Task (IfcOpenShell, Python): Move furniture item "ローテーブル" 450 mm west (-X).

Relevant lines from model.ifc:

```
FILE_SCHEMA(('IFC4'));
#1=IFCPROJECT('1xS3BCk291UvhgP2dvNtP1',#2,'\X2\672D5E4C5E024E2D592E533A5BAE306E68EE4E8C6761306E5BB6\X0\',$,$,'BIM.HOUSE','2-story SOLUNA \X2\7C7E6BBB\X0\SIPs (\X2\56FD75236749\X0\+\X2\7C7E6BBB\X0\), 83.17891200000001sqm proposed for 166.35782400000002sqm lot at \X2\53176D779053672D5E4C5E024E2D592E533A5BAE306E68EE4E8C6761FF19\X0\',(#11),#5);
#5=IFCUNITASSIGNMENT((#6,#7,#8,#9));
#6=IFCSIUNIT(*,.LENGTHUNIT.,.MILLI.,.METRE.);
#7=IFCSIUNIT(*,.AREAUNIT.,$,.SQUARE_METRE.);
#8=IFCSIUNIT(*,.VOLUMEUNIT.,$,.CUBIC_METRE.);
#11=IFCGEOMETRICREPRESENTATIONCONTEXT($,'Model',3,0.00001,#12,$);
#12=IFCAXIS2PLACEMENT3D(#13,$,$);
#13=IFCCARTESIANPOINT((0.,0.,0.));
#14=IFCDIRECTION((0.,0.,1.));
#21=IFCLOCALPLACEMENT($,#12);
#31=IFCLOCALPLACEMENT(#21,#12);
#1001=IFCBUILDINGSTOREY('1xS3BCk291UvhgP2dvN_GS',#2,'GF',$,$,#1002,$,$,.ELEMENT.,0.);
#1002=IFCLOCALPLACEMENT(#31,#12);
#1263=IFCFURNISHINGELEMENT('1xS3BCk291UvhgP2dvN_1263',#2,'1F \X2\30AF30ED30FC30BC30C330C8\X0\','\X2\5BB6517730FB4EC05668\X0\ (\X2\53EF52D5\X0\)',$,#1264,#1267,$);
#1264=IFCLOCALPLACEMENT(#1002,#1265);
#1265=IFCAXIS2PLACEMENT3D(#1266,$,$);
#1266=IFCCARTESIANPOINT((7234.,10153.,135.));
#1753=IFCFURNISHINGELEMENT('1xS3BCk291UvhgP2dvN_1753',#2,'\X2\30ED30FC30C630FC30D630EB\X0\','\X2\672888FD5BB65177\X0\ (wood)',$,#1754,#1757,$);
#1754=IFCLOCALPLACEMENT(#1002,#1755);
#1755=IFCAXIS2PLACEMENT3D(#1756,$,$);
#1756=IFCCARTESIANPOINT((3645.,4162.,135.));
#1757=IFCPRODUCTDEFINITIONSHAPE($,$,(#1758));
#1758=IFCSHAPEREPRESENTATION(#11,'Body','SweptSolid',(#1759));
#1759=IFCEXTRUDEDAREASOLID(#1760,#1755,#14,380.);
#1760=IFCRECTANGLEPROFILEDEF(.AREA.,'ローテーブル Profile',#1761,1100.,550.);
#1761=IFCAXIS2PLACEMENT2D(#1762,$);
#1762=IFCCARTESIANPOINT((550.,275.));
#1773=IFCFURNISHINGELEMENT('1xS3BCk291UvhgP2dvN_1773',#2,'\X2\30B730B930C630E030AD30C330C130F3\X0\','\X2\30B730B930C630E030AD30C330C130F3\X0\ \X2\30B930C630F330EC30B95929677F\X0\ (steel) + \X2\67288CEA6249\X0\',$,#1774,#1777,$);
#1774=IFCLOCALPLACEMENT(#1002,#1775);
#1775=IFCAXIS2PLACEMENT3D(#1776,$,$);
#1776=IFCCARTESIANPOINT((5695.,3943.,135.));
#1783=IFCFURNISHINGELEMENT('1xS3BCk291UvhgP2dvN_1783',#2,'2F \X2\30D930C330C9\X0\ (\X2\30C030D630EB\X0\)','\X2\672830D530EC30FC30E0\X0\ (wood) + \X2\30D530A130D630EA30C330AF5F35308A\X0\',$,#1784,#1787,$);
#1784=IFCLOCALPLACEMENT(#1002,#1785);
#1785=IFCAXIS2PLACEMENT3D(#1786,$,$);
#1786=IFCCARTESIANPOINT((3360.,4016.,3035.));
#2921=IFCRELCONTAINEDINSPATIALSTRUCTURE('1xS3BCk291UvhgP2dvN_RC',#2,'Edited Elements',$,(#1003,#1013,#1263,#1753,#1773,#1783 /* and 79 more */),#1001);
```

```python
import ifcopenshell
import ifcopenshell.api.geometry
import ifcopenshell.util.placement
import ifcopenshell.util.unit

model = ifcopenshell.open("model.ifc")
unit_scale = ifcopenshell.util.unit.calculate_unit_scale(model)

item = model.by_guid("1xS3BCk291UvhgP2dvN_1753")
matrix = ifcopenshell.util.placement.get_local_placement(item.ObjectPlacement)
matrix[0, 3] -= 0.45 / unit_scale
ifcopenshell.api.geometry.edit_object_placement(model, product=item, matrix=matrix, is_si=False)

print(ifcopenshell.util.placement.get_local_placement(item.ObjectPlacement).round(3) + 0.0)

model.write("model-out.ifc")
```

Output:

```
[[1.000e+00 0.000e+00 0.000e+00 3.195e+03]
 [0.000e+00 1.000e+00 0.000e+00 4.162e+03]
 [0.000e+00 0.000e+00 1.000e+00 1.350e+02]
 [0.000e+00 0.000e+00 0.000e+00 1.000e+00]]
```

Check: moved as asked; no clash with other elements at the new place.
